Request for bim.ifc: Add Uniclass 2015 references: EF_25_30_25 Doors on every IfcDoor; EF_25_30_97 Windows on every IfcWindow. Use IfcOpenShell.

First a look at what the model holds.

```python
import ifcopenshell

model = ifcopenshell.open("bim.ifc")
print(model.schema)
print("classifications:", [c.Name for c in model.by_type("IfcClassification")])
for ifc_class in ("IfcDoor", "IfcRoof", "IfcStair", "IfcWall", "IfcWindow"):
    print(ifc_class, len(model.by_type(ifc_class)))
```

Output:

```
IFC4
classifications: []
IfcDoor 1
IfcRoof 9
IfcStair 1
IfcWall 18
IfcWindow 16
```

```python
import ifcopenshell
import ifcopenshell.api.classification

model = ifcopenshell.open("bim.ifc")

system = ifcopenshell.api.classification.add_classification(model, classification="Uniclass 2015")

codes = {
    "IfcDoor": ("EF_25_30_25", "Doors"),
    "IfcWindow": ("EF_25_30_97", "Windows"),
}
for ifc_class, (code, name) in codes.items():
    products = model.by_type(ifc_class)
    ifcopenshell.api.classification.add_reference(
        model, products=products, classification=system, identification=code, name=name
    )
    print(code, len(products))

model.write("bim-out.ifc")
```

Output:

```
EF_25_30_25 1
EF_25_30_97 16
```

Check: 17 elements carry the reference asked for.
